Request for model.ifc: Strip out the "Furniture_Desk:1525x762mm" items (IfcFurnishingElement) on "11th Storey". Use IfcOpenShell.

First a look at what the model holds.

```python
import ifcopenshell
import ifcopenshell.util.element

model = ifcopenshell.open("model.ifc")
print(model.schema)
storey = next(s for s in model.by_type("IfcBuildingStorey") if s.Name == "11th Storey")
furniture = [e for e in ifcopenshell.util.element.get_decomposition(storey) if e.is_a("IfcFurnishingElement")]
seen = {}
for e in furniture:
    element_type = ifcopenshell.util.element.get_type(e)
    name = element_type.Name if element_type not in (None, e) else None
    seen[name] = seen.get(name, 0) + 1
for name, count in sorted(seen.items(), key=str):
    print(count, "x", name)
```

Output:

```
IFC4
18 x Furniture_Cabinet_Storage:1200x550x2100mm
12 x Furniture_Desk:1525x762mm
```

```python
import ifcopenshell
import ifcopenshell.api.root
import ifcopenshell.util.element

model = ifcopenshell.open("model.ifc")

storey = next(s for s in model.by_type("IfcBuildingStorey") if s.Name == "11th Storey")
furniture = [e for e in ifcopenshell.util.element.get_decomposition(storey) if e.is_a("IfcFurnishingElement")]
targets = [e for e in furniture if (t := ifcopenshell.util.element.get_type(e)) not in (None, e) and t.Name == "Furniture_Desk:1525x762mm"]

for e in targets:
    ifcopenshell.api.root.remove_product(model, product=e)
print(len(targets), "removed")

model.write("model_updated.ifc")
```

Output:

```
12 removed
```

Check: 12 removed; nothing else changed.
